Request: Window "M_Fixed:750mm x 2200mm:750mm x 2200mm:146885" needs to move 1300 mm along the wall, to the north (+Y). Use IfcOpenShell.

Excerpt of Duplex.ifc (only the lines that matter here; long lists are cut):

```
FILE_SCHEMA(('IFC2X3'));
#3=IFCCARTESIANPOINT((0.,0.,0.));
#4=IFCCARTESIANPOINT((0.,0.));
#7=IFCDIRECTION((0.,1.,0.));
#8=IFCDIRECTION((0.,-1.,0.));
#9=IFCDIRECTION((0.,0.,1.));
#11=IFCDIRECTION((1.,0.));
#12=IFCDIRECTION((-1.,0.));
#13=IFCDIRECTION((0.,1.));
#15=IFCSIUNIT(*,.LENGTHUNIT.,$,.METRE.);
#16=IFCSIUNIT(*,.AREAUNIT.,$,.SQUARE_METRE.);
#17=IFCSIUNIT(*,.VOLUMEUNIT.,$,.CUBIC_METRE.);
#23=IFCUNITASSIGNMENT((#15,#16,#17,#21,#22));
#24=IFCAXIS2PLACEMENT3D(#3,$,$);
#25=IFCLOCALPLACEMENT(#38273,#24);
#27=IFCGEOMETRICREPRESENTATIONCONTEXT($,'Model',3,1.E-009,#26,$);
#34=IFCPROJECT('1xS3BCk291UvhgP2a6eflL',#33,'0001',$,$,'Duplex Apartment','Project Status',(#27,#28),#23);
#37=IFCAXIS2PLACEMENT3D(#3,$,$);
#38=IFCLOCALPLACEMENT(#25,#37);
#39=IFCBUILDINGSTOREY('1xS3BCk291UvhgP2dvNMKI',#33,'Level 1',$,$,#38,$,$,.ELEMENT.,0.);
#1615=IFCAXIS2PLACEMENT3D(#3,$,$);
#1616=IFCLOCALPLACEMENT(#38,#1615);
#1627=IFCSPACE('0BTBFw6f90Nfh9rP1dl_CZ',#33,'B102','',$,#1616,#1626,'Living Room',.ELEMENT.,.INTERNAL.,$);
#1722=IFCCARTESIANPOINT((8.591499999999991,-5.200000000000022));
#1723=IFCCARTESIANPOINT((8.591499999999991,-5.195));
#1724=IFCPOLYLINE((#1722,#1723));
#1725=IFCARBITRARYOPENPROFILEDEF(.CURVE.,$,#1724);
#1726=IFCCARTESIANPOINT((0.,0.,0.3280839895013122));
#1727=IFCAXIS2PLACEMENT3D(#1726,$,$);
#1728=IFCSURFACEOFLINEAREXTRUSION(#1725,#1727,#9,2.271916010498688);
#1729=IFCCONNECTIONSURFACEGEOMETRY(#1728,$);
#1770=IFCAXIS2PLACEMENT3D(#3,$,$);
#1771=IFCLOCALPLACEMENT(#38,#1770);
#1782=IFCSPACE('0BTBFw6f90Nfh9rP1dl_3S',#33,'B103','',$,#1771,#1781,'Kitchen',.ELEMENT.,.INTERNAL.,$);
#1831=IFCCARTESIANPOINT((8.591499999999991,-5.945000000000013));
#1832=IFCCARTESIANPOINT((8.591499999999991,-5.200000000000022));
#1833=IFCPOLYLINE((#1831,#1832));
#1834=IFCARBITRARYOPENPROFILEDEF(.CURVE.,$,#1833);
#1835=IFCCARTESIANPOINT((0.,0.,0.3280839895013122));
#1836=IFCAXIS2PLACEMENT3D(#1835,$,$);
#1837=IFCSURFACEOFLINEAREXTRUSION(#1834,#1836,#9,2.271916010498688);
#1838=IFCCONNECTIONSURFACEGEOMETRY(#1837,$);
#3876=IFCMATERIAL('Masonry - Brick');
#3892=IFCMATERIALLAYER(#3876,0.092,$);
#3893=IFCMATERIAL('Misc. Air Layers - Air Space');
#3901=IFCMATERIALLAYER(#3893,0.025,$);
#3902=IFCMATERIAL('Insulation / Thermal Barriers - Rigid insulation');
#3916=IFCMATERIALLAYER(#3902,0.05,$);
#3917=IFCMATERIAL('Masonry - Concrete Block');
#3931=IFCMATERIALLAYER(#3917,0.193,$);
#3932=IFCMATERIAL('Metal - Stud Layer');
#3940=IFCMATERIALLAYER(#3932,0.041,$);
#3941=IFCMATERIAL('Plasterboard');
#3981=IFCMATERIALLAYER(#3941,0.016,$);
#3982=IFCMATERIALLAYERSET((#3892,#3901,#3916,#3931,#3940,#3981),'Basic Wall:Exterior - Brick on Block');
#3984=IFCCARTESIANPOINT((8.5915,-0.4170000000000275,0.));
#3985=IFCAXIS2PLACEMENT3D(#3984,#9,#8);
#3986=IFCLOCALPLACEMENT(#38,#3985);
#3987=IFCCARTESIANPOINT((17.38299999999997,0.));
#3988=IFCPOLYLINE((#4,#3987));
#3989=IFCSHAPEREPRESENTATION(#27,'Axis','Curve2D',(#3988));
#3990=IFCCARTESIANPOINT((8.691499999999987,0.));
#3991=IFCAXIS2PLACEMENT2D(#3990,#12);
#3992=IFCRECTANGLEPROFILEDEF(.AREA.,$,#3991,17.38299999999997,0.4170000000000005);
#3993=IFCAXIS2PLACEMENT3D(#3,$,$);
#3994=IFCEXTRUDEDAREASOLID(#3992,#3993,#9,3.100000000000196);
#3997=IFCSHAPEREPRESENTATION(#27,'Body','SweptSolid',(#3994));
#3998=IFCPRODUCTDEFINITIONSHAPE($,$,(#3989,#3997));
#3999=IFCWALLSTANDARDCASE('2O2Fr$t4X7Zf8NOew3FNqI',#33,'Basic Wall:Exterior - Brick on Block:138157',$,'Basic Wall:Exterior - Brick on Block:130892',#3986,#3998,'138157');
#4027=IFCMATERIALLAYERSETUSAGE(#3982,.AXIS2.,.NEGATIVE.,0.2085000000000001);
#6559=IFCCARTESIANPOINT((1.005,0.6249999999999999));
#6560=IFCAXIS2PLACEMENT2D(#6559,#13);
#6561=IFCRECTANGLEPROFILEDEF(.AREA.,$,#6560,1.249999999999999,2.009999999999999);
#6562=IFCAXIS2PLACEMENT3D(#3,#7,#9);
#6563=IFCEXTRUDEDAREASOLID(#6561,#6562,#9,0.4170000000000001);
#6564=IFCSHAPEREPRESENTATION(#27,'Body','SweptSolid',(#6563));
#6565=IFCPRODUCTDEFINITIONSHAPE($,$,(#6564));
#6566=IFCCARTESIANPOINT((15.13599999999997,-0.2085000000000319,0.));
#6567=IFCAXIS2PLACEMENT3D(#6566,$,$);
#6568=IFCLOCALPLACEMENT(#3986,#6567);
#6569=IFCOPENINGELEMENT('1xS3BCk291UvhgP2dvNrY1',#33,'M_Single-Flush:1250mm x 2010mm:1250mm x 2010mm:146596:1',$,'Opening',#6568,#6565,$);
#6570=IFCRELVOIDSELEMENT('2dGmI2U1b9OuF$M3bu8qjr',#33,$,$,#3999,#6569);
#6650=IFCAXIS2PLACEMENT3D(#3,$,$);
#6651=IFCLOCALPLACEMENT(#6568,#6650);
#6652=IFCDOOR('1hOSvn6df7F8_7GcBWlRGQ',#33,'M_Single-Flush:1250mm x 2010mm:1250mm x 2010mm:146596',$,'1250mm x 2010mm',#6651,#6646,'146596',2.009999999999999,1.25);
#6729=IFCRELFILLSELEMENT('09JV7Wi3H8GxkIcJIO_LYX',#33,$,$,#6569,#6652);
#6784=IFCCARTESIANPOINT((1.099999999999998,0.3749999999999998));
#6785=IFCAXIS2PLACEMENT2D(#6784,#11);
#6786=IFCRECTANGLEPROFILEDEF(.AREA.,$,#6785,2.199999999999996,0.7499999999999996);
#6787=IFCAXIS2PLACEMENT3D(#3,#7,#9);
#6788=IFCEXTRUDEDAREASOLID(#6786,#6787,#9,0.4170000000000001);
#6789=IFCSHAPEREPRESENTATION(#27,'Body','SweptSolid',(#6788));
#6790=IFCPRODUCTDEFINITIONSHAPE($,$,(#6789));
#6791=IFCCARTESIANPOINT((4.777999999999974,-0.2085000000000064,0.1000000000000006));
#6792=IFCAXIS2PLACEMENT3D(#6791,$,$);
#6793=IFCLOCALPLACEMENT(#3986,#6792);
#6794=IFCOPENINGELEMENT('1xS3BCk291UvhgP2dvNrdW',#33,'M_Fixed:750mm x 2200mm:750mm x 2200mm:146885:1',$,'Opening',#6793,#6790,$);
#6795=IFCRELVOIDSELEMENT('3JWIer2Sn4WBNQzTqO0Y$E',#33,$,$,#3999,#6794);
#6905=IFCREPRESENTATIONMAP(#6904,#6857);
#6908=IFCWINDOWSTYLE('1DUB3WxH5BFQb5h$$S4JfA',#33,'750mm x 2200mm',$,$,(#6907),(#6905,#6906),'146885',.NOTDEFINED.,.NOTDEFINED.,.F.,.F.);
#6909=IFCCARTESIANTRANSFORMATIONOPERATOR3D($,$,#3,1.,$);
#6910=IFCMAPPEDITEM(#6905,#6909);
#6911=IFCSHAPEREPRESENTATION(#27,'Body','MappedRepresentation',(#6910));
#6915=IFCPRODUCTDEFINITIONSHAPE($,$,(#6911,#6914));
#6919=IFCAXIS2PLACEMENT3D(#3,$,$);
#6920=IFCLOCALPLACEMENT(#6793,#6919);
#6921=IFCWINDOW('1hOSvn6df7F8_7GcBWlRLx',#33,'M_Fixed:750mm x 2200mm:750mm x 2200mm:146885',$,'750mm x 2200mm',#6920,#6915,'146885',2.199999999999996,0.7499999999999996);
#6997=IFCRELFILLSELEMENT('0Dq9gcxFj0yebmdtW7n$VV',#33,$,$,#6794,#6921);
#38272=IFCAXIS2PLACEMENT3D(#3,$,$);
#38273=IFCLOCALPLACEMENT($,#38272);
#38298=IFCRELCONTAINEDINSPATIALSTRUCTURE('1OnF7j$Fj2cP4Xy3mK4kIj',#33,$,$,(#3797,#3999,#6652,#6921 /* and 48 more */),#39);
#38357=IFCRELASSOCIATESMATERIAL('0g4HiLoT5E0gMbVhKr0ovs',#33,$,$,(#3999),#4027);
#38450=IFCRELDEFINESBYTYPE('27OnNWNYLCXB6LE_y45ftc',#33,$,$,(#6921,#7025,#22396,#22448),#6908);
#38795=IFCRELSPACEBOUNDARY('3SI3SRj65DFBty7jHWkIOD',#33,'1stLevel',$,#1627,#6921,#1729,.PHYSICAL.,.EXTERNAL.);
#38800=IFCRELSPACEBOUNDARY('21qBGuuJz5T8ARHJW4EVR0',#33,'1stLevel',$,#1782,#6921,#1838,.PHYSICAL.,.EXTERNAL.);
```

```python
import numpy as np
import ifcopenshell
import ifcopenshell.api.geometry
import ifcopenshell.util.placement
import ifcopenshell.util.unit

model = ifcopenshell.open("Duplex.ifc")
unit_scale = ifcopenshell.util.unit.calculate_unit_scale(model)

window = model.by_guid("1hOSvn6df7F8_7GcBWlRLx")
opening = window.FillsVoids[0].RelatingOpeningElement
wall = opening.VoidsElements[0].RelatingBuildingElement

wall_matrix = ifcopenshell.util.placement.get_local_placement(wall.ObjectPlacement)
shift = wall_matrix[:3, 0] * -1.3 / unit_scale
before = ifcopenshell.util.placement.get_local_placement(window.ObjectPlacement)[:3, 3].copy()

# The window is placed relative to its opening, so it follows when the opening moves.
matrix = ifcopenshell.util.placement.get_local_placement(opening.ObjectPlacement)
matrix[:3, 3] += shift
ifcopenshell.api.geometry.edit_object_placement(
    model, product=opening, matrix=matrix, is_si=False, should_transform_children=True
)

# Space boundary surfaces are stored in each space's coordinates; move them too.
for rel in window.ProvidesBoundaries:
    if not rel.ConnectionGeometry:
        continue
    surface = rel.ConnectionGeometry.SurfaceOnRelatingElement
    space_matrix = ifcopenshell.util.placement.get_local_placement(rel.RelatingSpace.ObjectPlacement)
    point = np.array(surface.Position.Location.Coordinates) + space_matrix[:3, :3].T @ shift
    surface.Position = model.createIfcAxis2Placement3D(
        model.createIfcCartesianPoint(point.tolist()), surface.Position.Axis, surface.Position.RefDirection
    )

after = ifcopenshell.util.placement.get_local_placement(window.ObjectPlacement)[:3, 3]
print("window moved by", (after - before).round(3) + 0.0)

model.write("Duplex_edited.ifc")
```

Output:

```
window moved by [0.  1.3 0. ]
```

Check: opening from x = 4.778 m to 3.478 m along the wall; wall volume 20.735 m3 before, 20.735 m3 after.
